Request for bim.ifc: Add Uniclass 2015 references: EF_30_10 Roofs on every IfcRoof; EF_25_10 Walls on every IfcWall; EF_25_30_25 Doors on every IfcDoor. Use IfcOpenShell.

First a look at what the model holds.

```python
import ifcopenshell

model = ifcopenshell.open("bim.ifc")
print(model.schema)
print("classifications:", [c.Name for c in model.by_type("IfcClassification")])
for ifc_class in ("IfcDoor", "IfcRoof", "IfcStair", "IfcWall", "IfcWindow"):
    print(ifc_class, len(model.by_type(ifc_class)))
```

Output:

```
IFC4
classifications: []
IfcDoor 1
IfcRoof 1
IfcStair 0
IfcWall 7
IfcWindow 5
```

```python
import ifcopenshell
import ifcopenshell.api.classification

model = ifcopenshell.open("bim.ifc")

system = ifcopenshell.api.classification.add_classification(model, classification="Uniclass 2015")

codes = {
    "IfcRoof": ("EF_30_10", "Roofs"),
    "IfcWall": ("EF_25_10", "Walls"),
    "IfcDoor": ("EF_25_30_25", "Doors"),
}
for ifc_class, (code, name) in codes.items():
    products = model.by_type(ifc_class)
    ifcopenshell.api.classification.add_reference(
        model, products=products, classification=system, identification=code, name=name
    )
    print(code, len(products))

model.write("bim_rev.ifc")
```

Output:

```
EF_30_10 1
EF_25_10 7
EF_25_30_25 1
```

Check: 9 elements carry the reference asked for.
